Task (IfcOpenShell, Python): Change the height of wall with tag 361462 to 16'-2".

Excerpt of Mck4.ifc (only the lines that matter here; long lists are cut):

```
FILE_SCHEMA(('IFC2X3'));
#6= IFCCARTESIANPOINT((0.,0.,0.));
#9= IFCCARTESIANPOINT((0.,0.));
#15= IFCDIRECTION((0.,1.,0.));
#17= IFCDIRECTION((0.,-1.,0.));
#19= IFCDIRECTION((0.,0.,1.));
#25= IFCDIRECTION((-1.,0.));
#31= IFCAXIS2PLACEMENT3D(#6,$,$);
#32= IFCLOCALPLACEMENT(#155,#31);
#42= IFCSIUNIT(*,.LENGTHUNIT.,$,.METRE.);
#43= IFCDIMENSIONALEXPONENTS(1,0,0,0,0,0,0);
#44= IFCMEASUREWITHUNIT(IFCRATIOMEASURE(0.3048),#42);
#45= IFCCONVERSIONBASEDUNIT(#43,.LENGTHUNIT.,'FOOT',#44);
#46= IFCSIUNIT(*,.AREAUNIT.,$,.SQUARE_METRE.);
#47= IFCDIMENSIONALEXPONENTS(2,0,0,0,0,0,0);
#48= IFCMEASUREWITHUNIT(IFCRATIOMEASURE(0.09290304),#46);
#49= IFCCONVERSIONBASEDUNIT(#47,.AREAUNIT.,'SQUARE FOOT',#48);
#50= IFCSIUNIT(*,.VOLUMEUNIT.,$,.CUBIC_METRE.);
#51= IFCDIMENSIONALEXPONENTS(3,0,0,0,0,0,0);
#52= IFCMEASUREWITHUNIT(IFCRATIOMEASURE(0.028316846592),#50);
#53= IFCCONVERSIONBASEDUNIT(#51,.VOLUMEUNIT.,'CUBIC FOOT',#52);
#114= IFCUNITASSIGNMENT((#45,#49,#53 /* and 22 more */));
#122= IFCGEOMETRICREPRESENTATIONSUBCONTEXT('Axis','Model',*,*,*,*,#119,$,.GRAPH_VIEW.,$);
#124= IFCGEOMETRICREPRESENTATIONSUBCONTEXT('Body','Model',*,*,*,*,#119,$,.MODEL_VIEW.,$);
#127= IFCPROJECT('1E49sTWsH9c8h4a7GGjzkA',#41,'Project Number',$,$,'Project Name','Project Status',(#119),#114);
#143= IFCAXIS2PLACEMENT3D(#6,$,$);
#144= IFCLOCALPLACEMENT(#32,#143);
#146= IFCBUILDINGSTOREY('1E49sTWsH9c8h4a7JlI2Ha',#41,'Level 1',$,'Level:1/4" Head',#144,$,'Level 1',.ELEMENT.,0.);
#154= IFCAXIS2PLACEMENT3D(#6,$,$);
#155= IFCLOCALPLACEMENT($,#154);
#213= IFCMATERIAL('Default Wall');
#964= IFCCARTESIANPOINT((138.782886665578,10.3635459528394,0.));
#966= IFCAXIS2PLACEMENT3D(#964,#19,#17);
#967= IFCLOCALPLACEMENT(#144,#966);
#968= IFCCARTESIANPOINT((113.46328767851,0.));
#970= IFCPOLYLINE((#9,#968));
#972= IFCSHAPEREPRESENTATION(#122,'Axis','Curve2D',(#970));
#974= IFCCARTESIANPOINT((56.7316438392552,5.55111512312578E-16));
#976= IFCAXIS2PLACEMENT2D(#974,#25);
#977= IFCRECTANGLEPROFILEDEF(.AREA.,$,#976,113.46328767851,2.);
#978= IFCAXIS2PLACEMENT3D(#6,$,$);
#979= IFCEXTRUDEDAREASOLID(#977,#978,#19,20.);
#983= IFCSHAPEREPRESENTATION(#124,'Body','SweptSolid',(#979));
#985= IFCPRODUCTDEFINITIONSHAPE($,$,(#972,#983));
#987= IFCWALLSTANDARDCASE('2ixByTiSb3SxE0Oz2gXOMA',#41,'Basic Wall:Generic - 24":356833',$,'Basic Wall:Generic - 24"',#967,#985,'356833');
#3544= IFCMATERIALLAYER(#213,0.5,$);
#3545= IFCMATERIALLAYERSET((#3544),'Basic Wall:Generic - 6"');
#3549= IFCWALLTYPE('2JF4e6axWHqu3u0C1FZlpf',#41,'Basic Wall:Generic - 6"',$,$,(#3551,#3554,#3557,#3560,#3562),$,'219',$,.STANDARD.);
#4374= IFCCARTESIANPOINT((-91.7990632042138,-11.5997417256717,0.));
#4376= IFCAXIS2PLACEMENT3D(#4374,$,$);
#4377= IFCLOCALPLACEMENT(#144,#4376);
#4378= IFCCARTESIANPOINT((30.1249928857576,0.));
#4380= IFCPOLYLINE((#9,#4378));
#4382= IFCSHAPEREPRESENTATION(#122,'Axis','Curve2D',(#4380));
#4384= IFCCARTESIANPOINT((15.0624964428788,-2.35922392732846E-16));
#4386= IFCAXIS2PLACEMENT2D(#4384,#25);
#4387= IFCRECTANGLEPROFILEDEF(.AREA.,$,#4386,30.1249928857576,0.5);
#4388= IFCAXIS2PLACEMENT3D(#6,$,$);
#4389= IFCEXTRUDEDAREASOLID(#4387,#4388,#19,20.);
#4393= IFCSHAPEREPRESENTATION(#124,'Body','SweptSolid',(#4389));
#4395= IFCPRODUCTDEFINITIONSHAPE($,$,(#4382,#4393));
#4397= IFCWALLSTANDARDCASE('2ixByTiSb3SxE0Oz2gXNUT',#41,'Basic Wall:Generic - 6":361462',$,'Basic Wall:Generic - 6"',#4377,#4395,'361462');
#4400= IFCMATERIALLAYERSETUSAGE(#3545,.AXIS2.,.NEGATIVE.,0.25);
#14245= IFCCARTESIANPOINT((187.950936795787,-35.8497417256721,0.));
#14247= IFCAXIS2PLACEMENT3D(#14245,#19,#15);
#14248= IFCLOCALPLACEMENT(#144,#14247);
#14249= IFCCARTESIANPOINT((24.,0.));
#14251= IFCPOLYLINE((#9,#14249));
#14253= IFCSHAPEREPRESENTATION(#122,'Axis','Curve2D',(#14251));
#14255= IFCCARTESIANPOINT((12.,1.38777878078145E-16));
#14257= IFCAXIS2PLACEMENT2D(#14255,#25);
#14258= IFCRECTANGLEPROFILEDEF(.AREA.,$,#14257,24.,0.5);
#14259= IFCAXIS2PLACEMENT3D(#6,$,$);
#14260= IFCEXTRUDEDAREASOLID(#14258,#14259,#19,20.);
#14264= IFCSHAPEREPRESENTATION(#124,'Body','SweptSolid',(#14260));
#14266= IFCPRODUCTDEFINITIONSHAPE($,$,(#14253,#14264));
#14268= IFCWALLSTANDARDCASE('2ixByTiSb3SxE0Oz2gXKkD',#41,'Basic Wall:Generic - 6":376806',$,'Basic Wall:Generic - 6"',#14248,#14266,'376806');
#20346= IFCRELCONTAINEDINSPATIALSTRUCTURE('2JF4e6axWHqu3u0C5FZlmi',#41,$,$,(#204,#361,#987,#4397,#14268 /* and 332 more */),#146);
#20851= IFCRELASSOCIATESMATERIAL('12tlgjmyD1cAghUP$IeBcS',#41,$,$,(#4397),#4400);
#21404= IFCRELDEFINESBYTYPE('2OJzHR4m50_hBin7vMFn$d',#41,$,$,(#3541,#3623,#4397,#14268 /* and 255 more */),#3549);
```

```python
import ifcopenshell
import ifcopenshell.geom
import ifcopenshell.util.representation
import ifcopenshell.util.shape
import ifcopenshell.util.unit

model = ifcopenshell.open("Mck4.ifc")
unit_scale = ifcopenshell.util.unit.calculate_unit_scale(model)
settings = ifcopenshell.geom.settings()


def volume(element):
    """Net volume in cubic metres, openings subtracted."""
    shape = ifcopenshell.geom.create_shape(settings, element)
    return ifcopenshell.util.shape.get_volume(shape.geometry)


wall = model.by_guid("2ixByTiSb3SxE0Oz2gXNUT")
before = volume(wall)

body = ifcopenshell.util.representation.get_representation(wall, "Model", "Body")
solid = body.Items[0]
old_height = solid.Depth
solid.Depth = 194 * 0.0254 / unit_scale
after = volume(wall)

print(f"height {old_height:g} -> {solid.Depth:g}, volume {before:.3f} -> {after:.3f} m3")

model.write("Mck4_edited.ifc")
```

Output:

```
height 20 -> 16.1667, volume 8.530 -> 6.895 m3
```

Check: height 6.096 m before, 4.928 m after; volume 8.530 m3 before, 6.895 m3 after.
